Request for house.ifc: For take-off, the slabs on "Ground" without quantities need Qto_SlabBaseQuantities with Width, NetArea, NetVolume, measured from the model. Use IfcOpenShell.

First a look at what the model holds.

```python
import ifcopenshell
import ifcopenshell.util.element
import ifcopenshell.util.unit

model = ifcopenshell.open("house.ifc")
print(model.schema)
for unit_type in ("LENGTHUNIT", "AREAUNIT", "VOLUMEUNIT"):
    print(unit_type, ifcopenshell.util.unit.calculate_unit_scale(model, unit_type))
storey = next(s for s in model.by_type("IfcBuildingStorey") if s.Name == "Ground")
slabs = [e for e in ifcopenshell.util.element.get_decomposition(storey) if e.is_a("IfcSlab")]
for e in sorted(slabs, key=lambda e: e.id()):
    print(e.id(), e.is_a(), e.Name, list(ifcopenshell.util.element.get_psets(e, qtos_only=True)), sep=" | ")
```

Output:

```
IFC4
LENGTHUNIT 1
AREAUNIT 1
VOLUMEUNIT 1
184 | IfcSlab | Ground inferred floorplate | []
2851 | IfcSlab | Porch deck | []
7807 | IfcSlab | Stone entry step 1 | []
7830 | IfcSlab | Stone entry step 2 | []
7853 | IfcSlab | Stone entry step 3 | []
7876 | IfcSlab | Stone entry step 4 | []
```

```python
import ifcopenshell
import ifcopenshell.api.pset
import ifcopenshell.geom
import ifcopenshell.util.element
import ifcopenshell.util.shape
import ifcopenshell.util.unit

model = ifcopenshell.open("house.ifc")
unit_scale = ifcopenshell.util.unit.calculate_unit_scale(model)
area_scale = ifcopenshell.util.unit.calculate_unit_scale(model, "AREAUNIT")
volume_scale = ifcopenshell.util.unit.calculate_unit_scale(model, "VOLUMEUNIT")
settings = ifcopenshell.geom.settings()

storey = next(s for s in model.by_type("IfcBuildingStorey") if s.Name == "Ground")
slabs = [e for e in ifcopenshell.util.element.get_decomposition(storey) if e.is_a("IfcSlab")]

for e in sorted(slabs, key=lambda e: e.id()):
    if ifcopenshell.util.element.get_psets(e, qtos_only=True, should_inherit=False):
        continue
    # Geometry comes back in metres, in the element's own axes.
    shape = ifcopenshell.geom.create_shape(settings, e)
    values = {
        "Width": ifcopenshell.util.shape.get_z(shape.geometry) / unit_scale,
        "NetArea": ifcopenshell.util.shape.get_footprint_area(shape.geometry) / area_scale,
        "NetVolume": ifcopenshell.util.shape.get_volume(shape.geometry) / volume_scale,
    }
    qto = ifcopenshell.api.pset.add_qto(model, product=e, name="Qto_SlabBaseQuantities")
    ifcopenshell.api.pset.edit_qto(model, qto=qto, properties=values)
    print(e.id(), {k: round(v, 3) for k, v in values.items()})

model.write("house_rev.ifc")
```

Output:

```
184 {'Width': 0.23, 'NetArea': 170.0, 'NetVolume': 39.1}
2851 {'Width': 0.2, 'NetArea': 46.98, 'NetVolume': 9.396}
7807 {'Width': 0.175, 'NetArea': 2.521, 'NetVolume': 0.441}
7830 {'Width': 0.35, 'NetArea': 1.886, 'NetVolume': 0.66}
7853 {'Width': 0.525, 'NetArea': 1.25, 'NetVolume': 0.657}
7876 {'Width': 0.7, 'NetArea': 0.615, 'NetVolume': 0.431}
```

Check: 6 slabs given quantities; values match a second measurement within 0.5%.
